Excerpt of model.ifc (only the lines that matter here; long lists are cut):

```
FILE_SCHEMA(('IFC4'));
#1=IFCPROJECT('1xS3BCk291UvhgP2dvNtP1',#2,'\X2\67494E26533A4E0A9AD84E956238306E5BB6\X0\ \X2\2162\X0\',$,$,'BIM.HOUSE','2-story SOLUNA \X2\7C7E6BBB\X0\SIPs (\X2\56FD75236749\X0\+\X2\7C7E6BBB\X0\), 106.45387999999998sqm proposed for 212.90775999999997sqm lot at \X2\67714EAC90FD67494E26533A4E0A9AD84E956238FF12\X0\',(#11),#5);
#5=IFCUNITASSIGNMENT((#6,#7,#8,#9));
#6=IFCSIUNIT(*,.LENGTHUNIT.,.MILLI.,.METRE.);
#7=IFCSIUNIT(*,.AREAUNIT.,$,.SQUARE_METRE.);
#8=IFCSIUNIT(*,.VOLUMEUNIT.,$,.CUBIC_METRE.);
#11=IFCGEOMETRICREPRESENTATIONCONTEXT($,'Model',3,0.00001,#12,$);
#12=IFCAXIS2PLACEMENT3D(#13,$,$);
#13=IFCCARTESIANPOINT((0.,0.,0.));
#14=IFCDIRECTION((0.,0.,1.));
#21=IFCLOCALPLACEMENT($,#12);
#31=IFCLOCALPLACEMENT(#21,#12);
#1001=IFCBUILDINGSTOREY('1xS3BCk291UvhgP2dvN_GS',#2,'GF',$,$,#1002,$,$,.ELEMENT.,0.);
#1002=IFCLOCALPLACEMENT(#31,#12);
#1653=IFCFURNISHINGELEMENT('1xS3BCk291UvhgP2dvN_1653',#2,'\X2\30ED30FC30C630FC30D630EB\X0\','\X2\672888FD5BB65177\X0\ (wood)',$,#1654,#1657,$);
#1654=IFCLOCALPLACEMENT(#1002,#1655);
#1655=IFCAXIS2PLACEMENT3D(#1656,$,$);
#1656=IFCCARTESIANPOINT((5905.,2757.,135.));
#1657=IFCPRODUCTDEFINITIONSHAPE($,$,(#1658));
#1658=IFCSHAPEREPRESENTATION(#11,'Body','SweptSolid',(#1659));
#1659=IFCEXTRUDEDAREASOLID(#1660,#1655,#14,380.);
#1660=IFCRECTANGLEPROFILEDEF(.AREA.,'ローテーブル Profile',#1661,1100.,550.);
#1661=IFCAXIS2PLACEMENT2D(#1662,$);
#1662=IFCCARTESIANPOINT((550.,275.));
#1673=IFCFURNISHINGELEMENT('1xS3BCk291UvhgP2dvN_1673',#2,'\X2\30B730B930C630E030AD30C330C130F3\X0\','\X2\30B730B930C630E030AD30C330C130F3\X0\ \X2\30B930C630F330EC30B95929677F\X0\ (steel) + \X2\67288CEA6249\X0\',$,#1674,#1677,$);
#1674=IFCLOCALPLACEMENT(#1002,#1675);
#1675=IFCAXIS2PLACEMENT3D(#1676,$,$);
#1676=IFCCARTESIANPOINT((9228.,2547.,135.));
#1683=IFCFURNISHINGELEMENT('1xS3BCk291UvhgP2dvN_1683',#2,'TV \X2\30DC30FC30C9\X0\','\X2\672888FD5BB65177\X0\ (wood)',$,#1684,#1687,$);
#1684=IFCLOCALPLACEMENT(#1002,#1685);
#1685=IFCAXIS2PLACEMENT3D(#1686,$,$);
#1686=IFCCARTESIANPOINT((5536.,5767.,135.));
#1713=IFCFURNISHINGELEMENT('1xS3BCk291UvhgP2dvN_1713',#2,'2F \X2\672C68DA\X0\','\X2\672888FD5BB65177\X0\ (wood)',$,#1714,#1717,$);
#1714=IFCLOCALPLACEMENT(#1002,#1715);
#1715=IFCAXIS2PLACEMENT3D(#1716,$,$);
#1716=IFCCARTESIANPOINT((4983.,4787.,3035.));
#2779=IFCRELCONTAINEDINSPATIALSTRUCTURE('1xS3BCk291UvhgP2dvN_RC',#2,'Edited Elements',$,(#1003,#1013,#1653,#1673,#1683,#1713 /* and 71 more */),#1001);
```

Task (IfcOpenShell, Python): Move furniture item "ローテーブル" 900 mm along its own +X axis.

```python
import ifcopenshell
import ifcopenshell.api.geometry
import ifcopenshell.util.placement
import ifcopenshell.util.unit

model = ifcopenshell.open("model.ifc")
unit_scale = ifcopenshell.util.unit.calculate_unit_scale(model)

item = model.by_id(1653)
matrix = ifcopenshell.util.placement.get_local_placement(item.ObjectPlacement)
matrix[:3, 3] += matrix[:3, 0] * 0.9 / unit_scale
ifcopenshell.api.geometry.edit_object_placement(model, product=item, matrix=matrix, is_si=False)

print(ifcopenshell.util.placement.get_local_placement(item.ObjectPlacement).round(3) + 0.0)

model.write("model_edited.ifc")
```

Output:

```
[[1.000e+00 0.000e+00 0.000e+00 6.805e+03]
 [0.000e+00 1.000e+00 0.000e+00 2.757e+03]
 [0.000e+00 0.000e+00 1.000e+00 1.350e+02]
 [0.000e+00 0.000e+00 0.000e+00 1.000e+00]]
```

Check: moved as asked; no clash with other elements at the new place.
